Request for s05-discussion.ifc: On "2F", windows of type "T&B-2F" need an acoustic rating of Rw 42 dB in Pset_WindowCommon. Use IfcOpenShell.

First a look at what the model holds.

```python
import ifcopenshell
import ifcopenshell.util.element

model = ifcopenshell.open("s05-discussion.ifc")
print(model.schema)
storey = next(s for s in model.by_type("IfcBuildingStorey") if s.Name == "2F")
windows = [e for e in ifcopenshell.util.element.get_decomposition(storey) if e.is_a("IfcWindow")]
seen = {}
for e in windows:
    element_type = ifcopenshell.util.element.get_type(e)
    key = (element_type.Name if element_type != e and element_type else None, ifcopenshell.util.element.get_pset(e, "Pset_WindowCommon", "AcousticRating"))
    seen[key] = seen.get(key, 0) + 1
for (name, value), count in sorted(seen.items(), key=str):
    print(count, "x", name, "|", value)
```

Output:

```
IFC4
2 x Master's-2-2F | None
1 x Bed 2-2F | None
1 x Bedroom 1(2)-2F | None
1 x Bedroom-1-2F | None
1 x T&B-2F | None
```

```python
import ifcopenshell
import ifcopenshell.api.pset
import ifcopenshell.util.element

model = ifcopenshell.open("s05-discussion.ifc")

storey = next(s for s in model.by_type("IfcBuildingStorey") if s.Name == "2F")
windows = [e for e in ifcopenshell.util.element.get_decomposition(storey) if e.is_a("IfcWindow")]

count = 0
for e in windows:
    element_type = ifcopenshell.util.element.get_type(e)
    if element_type in (None, e) or element_type.Name != "T&B-2F":
        continue
    # add_pset returns the element's existing set when there is one.
    pset = ifcopenshell.api.pset.add_pset(model, product=e, name="Pset_WindowCommon")
    ifcopenshell.api.pset.edit_pset(model, pset=pset, properties={"AcousticRating": "Rw 42 dB"})
    count += 1

print(count, "windows updated")

model.write("s05-discussion_rev.ifc")
```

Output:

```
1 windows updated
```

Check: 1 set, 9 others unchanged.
